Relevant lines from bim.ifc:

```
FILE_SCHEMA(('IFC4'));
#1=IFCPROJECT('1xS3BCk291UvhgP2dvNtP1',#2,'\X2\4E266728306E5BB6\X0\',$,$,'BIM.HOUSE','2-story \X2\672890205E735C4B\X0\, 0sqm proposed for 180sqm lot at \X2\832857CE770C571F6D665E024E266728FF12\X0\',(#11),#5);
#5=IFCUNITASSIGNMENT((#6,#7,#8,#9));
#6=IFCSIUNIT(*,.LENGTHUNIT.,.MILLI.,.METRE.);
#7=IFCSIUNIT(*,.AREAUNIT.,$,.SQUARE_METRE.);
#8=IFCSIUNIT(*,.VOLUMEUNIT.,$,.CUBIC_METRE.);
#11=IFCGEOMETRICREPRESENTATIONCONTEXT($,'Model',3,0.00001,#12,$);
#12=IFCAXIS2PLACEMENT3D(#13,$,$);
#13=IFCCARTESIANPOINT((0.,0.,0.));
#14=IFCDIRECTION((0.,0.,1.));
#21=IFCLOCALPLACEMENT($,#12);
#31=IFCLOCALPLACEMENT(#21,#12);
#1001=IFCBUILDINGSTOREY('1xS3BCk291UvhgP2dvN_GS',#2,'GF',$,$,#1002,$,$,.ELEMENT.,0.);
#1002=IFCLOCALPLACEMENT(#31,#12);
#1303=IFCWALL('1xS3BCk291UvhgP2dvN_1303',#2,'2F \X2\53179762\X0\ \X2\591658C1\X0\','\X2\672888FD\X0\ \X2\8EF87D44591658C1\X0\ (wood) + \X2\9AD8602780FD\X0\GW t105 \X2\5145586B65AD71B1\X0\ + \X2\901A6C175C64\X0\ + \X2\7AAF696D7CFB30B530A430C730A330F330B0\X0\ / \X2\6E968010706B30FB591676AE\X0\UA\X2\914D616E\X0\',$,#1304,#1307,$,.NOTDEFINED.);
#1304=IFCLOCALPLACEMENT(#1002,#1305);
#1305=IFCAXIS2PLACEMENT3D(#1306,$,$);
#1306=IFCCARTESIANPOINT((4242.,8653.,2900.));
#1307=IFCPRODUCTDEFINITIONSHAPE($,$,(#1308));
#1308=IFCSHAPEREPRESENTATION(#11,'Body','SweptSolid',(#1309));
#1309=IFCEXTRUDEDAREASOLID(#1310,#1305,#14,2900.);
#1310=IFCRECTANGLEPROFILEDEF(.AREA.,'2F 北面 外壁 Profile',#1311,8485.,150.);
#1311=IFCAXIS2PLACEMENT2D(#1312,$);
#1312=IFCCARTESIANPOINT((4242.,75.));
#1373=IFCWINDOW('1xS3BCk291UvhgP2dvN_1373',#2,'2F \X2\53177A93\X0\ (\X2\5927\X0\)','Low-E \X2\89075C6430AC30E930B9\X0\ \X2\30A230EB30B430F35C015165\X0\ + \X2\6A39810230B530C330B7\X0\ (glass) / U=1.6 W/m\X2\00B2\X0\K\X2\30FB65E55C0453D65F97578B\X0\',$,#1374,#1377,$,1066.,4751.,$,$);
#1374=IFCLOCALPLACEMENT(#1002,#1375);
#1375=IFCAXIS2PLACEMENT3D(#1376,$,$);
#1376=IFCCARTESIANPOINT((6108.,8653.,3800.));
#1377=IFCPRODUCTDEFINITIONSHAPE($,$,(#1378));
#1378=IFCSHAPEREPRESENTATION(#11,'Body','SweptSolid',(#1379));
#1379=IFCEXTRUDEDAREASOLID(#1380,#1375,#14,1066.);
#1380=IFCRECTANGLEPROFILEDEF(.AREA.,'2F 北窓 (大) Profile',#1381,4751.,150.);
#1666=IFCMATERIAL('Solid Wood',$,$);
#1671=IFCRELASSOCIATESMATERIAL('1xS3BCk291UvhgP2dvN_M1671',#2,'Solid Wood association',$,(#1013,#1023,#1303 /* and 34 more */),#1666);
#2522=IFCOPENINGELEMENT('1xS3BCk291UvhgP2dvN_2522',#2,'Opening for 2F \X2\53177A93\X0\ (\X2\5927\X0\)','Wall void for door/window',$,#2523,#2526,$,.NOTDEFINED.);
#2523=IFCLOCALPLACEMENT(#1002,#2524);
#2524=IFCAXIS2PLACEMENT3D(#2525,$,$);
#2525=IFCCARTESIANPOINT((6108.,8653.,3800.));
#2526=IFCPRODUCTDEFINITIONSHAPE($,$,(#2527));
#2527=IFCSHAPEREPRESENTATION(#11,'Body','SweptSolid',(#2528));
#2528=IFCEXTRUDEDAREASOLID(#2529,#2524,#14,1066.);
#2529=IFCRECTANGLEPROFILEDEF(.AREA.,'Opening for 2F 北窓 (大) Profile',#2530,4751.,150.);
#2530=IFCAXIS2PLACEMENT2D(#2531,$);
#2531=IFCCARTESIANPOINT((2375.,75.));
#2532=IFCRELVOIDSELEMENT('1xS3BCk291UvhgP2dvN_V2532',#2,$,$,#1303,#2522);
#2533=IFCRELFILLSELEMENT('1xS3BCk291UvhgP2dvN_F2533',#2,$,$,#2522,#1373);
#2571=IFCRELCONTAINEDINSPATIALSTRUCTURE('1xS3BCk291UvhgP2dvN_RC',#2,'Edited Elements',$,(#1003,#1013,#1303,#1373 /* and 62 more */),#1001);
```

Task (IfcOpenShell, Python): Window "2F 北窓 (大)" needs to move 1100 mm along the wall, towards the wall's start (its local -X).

```python
import ifcopenshell
import ifcopenshell.api.geometry
import ifcopenshell.util.placement

model = ifcopenshell.open("bim.ifc")

window = model.by_id(1373)
opening = window.FillsVoids[0].RelatingOpeningElement
wall = opening.VoidsElements[0].RelatingBuildingElement

wall_matrix = ifcopenshell.util.placement.get_local_placement(wall.ObjectPlacement)
shift = wall_matrix[:3, 0] * -1100.0
before = ifcopenshell.util.placement.get_local_placement(window.ObjectPlacement)[:3, 3].copy()

# The window is not placed relative to its opening, so move both.
for product in (opening, window):
    matrix = ifcopenshell.util.placement.get_local_placement(product.ObjectPlacement)
    matrix[:3, 3] += shift
    ifcopenshell.api.geometry.edit_object_placement(model, product=product, matrix=matrix, is_si=False)

after = ifcopenshell.util.placement.get_local_placement(window.ObjectPlacement)[:3, 3]
print("window moved by", (after - before).round(3) + 0.0)

model.write("bim_edited.ifc")
```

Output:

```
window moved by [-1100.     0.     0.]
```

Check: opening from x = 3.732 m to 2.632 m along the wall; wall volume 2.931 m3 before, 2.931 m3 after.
